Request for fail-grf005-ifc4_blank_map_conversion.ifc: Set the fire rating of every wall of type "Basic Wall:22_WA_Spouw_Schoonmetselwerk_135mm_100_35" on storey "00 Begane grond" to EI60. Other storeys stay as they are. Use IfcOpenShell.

First a look at what the model holds.

```python
import ifcopenshell
import ifcopenshell.util.element

model = ifcopenshell.open("fail-grf005-ifc4_blank_map_conversion.ifc")
print(model.schema)
storey = next(s for s in model.by_type("IfcBuildingStorey") if s.Name == "00 Begane grond")
walls = [e for e in ifcopenshell.util.element.get_decomposition(storey) if e.is_a("IfcWall")]
seen = {}
for e in walls:
    element_type = ifcopenshell.util.element.get_type(e)
    key = (element_type.Name if element_type != e and element_type else None, ifcopenshell.util.element.get_pset(e, "Pset_WallCommon", "FireRating"))
    seen[key] = seen.get(key, 0) + 1
for (name, value), count in sorted(seen.items(), key=str):
    print(count, "x", name, "|", value)
```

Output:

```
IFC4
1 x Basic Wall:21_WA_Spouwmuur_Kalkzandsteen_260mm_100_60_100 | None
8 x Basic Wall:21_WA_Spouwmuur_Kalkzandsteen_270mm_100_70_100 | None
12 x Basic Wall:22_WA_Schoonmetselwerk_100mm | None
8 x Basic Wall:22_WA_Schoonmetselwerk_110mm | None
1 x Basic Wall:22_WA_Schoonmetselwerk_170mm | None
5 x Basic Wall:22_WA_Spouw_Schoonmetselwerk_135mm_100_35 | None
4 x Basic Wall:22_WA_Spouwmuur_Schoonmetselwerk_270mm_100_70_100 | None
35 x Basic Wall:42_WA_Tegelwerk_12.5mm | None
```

```python
import ifcopenshell
import ifcopenshell.api.pset
import ifcopenshell.util.element

model = ifcopenshell.open("fail-grf005-ifc4_blank_map_conversion.ifc")

storey = next(s for s in model.by_type("IfcBuildingStorey") if s.Name == "00 Begane grond")
walls = [e for e in ifcopenshell.util.element.get_decomposition(storey) if e.is_a("IfcWall")]

count = 0
for e in walls:
    element_type = ifcopenshell.util.element.get_type(e)
    if element_type in (None, e) or element_type.Name != "Basic Wall:22_WA_Spouw_Schoonmetselwerk_135mm_100_35":
        continue
    # add_pset returns the element's existing set when there is one.
    pset = ifcopenshell.api.pset.add_pset(model, product=e, name="Pset_WallCommon")
    ifcopenshell.api.pset.edit_pset(model, pset=pset, properties={"FireRating": "EI60"})
    count += 1

print(count, "walls updated")

model.write("fail-grf005-ifc4_blank_map_conversion_edited.ifc")
```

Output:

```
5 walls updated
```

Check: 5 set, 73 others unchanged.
